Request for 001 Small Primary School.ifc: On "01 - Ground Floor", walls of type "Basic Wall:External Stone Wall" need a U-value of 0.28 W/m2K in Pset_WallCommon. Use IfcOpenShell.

First a look at what the model holds.

```python
import ifcopenshell
import ifcopenshell.util.element

model = ifcopenshell.open("001 Small Primary School.ifc")
print(model.schema)
storey = next(s for s in model.by_type("IfcBuildingStorey") if s.Name == "01 - Ground Floor")
walls = [e for e in ifcopenshell.util.element.get_decomposition(storey) if e.is_a("IfcWall")]
seen = {}
for e in walls:
    element_type = ifcopenshell.util.element.get_type(e)
    key = (element_type.Name if element_type != e and element_type else None, ifcopenshell.util.element.get_pset(e, "Pset_WallCommon", "ThermalTransmittance"))
    seen[key] = seen.get(key, 0) + 1
for (name, value), count in sorted(seen.items(), key=str):
    print(count, "x", name, "|", value)
```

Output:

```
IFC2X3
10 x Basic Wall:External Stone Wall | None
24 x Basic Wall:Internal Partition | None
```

```python
import ifcopenshell
import ifcopenshell.api.pset
import ifcopenshell.util.element

model = ifcopenshell.open("001 Small Primary School.ifc")

storey = next(s for s in model.by_type("IfcBuildingStorey") if s.Name == "01 - Ground Floor")
walls = [e for e in ifcopenshell.util.element.get_decomposition(storey) if e.is_a("IfcWall")]

count = 0
for e in walls:
    element_type = ifcopenshell.util.element.get_type(e)
    if element_type in (None, e) or element_type.Name != "Basic Wall:External Stone Wall":
        continue
    # add_pset returns the element's existing set when there is one.
    pset = ifcopenshell.api.pset.add_pset(model, product=e, name="Pset_WallCommon")
    ifcopenshell.api.pset.edit_pset(model, pset=pset, properties={"ThermalTransmittance": 0.28})
    count += 1

print(count, "walls updated")

model.write("001 Small Primary School_v2.ifc")
```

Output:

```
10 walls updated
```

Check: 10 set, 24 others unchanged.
